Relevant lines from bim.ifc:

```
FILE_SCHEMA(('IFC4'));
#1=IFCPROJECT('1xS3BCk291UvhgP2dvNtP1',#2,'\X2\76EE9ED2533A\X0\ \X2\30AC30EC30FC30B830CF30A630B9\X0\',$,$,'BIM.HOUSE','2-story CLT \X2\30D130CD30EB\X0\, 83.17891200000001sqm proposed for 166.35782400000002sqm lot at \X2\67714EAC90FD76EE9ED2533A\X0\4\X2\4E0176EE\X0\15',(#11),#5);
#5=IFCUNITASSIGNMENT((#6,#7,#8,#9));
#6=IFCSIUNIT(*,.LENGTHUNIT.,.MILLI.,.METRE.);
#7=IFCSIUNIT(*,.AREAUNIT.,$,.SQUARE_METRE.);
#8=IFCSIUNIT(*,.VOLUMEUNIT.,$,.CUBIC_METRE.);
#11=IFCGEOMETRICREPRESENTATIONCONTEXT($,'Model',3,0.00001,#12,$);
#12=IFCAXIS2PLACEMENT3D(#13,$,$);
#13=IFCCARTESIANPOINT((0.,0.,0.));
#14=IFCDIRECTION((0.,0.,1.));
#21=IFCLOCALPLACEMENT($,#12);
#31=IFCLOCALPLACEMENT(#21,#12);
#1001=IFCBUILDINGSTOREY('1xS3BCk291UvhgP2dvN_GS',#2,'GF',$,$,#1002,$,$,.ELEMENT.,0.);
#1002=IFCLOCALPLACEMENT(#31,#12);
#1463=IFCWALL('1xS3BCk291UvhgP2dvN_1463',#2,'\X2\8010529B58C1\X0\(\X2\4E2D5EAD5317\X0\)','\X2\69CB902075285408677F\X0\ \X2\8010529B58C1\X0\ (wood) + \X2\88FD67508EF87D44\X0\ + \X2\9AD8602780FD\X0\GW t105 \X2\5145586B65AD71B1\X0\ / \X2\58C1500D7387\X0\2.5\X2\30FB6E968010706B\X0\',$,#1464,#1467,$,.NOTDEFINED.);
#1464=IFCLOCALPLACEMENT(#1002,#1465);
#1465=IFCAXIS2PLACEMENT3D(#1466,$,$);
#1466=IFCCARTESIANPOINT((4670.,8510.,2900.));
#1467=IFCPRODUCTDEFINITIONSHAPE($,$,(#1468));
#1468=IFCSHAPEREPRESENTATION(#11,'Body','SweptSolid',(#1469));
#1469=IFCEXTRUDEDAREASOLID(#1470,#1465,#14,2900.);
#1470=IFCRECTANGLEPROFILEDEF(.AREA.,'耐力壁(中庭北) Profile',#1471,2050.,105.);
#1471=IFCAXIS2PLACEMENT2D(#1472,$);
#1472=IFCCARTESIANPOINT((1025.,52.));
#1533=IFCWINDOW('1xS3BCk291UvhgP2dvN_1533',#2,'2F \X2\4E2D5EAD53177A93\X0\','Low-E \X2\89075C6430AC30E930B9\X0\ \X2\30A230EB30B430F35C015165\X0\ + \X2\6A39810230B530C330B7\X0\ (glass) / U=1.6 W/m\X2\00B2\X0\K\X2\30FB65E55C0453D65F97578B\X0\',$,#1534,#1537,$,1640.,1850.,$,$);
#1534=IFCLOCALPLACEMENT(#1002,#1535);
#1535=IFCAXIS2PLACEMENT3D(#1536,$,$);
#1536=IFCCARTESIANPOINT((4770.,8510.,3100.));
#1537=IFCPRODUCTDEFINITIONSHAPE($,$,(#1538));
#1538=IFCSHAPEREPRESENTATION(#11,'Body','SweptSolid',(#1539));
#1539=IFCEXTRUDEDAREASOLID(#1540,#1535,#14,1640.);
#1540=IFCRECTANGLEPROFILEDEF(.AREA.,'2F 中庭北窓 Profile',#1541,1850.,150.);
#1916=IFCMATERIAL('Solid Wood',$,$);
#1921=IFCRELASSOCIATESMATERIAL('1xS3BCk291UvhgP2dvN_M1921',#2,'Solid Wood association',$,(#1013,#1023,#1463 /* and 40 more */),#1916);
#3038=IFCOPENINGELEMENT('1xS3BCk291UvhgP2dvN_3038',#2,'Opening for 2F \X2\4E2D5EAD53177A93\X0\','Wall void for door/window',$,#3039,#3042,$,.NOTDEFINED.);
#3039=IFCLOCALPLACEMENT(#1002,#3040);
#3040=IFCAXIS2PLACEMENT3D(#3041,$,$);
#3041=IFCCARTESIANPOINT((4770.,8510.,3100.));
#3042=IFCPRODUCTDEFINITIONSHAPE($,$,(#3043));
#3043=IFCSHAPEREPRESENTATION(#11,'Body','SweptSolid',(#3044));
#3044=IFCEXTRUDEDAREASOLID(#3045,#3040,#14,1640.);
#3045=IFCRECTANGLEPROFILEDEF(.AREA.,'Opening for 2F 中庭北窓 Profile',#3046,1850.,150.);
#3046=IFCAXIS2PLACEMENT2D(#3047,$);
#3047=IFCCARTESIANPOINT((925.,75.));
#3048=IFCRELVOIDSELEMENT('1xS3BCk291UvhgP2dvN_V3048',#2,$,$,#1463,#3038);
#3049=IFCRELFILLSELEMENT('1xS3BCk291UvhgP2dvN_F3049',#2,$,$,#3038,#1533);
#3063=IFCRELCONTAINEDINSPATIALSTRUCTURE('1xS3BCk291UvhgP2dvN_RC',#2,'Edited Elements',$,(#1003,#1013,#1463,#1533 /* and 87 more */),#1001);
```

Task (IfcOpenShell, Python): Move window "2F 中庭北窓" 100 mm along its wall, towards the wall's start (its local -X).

```python
import ifcopenshell
import ifcopenshell.api.geometry
import ifcopenshell.util.placement

model = ifcopenshell.open("bim.ifc")

window = model.by_guid("1xS3BCk291UvhgP2dvN_1533")
opening = window.FillsVoids[0].RelatingOpeningElement
wall = opening.VoidsElements[0].RelatingBuildingElement

wall_matrix = ifcopenshell.util.placement.get_local_placement(wall.ObjectPlacement)
shift = wall_matrix[:3, 0] * -100.0
before = ifcopenshell.util.placement.get_local_placement(window.ObjectPlacement)[:3, 3].copy()

# The window is not placed relative to its opening, so move both.
for product in (opening, window):
    matrix = ifcopenshell.util.placement.get_local_placement(product.ObjectPlacement)
    matrix[:3, 3] += shift
    ifcopenshell.api.geometry.edit_object_placement(model, product=product, matrix=matrix, is_si=False)

after = ifcopenshell.util.placement.get_local_placement(window.ObjectPlacement)[:3, 3]
print("window moved by", (after - before).round(3) + 0.0)

model.write("bim_edited.ifc")
```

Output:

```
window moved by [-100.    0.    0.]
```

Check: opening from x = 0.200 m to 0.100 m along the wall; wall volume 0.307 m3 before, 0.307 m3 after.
